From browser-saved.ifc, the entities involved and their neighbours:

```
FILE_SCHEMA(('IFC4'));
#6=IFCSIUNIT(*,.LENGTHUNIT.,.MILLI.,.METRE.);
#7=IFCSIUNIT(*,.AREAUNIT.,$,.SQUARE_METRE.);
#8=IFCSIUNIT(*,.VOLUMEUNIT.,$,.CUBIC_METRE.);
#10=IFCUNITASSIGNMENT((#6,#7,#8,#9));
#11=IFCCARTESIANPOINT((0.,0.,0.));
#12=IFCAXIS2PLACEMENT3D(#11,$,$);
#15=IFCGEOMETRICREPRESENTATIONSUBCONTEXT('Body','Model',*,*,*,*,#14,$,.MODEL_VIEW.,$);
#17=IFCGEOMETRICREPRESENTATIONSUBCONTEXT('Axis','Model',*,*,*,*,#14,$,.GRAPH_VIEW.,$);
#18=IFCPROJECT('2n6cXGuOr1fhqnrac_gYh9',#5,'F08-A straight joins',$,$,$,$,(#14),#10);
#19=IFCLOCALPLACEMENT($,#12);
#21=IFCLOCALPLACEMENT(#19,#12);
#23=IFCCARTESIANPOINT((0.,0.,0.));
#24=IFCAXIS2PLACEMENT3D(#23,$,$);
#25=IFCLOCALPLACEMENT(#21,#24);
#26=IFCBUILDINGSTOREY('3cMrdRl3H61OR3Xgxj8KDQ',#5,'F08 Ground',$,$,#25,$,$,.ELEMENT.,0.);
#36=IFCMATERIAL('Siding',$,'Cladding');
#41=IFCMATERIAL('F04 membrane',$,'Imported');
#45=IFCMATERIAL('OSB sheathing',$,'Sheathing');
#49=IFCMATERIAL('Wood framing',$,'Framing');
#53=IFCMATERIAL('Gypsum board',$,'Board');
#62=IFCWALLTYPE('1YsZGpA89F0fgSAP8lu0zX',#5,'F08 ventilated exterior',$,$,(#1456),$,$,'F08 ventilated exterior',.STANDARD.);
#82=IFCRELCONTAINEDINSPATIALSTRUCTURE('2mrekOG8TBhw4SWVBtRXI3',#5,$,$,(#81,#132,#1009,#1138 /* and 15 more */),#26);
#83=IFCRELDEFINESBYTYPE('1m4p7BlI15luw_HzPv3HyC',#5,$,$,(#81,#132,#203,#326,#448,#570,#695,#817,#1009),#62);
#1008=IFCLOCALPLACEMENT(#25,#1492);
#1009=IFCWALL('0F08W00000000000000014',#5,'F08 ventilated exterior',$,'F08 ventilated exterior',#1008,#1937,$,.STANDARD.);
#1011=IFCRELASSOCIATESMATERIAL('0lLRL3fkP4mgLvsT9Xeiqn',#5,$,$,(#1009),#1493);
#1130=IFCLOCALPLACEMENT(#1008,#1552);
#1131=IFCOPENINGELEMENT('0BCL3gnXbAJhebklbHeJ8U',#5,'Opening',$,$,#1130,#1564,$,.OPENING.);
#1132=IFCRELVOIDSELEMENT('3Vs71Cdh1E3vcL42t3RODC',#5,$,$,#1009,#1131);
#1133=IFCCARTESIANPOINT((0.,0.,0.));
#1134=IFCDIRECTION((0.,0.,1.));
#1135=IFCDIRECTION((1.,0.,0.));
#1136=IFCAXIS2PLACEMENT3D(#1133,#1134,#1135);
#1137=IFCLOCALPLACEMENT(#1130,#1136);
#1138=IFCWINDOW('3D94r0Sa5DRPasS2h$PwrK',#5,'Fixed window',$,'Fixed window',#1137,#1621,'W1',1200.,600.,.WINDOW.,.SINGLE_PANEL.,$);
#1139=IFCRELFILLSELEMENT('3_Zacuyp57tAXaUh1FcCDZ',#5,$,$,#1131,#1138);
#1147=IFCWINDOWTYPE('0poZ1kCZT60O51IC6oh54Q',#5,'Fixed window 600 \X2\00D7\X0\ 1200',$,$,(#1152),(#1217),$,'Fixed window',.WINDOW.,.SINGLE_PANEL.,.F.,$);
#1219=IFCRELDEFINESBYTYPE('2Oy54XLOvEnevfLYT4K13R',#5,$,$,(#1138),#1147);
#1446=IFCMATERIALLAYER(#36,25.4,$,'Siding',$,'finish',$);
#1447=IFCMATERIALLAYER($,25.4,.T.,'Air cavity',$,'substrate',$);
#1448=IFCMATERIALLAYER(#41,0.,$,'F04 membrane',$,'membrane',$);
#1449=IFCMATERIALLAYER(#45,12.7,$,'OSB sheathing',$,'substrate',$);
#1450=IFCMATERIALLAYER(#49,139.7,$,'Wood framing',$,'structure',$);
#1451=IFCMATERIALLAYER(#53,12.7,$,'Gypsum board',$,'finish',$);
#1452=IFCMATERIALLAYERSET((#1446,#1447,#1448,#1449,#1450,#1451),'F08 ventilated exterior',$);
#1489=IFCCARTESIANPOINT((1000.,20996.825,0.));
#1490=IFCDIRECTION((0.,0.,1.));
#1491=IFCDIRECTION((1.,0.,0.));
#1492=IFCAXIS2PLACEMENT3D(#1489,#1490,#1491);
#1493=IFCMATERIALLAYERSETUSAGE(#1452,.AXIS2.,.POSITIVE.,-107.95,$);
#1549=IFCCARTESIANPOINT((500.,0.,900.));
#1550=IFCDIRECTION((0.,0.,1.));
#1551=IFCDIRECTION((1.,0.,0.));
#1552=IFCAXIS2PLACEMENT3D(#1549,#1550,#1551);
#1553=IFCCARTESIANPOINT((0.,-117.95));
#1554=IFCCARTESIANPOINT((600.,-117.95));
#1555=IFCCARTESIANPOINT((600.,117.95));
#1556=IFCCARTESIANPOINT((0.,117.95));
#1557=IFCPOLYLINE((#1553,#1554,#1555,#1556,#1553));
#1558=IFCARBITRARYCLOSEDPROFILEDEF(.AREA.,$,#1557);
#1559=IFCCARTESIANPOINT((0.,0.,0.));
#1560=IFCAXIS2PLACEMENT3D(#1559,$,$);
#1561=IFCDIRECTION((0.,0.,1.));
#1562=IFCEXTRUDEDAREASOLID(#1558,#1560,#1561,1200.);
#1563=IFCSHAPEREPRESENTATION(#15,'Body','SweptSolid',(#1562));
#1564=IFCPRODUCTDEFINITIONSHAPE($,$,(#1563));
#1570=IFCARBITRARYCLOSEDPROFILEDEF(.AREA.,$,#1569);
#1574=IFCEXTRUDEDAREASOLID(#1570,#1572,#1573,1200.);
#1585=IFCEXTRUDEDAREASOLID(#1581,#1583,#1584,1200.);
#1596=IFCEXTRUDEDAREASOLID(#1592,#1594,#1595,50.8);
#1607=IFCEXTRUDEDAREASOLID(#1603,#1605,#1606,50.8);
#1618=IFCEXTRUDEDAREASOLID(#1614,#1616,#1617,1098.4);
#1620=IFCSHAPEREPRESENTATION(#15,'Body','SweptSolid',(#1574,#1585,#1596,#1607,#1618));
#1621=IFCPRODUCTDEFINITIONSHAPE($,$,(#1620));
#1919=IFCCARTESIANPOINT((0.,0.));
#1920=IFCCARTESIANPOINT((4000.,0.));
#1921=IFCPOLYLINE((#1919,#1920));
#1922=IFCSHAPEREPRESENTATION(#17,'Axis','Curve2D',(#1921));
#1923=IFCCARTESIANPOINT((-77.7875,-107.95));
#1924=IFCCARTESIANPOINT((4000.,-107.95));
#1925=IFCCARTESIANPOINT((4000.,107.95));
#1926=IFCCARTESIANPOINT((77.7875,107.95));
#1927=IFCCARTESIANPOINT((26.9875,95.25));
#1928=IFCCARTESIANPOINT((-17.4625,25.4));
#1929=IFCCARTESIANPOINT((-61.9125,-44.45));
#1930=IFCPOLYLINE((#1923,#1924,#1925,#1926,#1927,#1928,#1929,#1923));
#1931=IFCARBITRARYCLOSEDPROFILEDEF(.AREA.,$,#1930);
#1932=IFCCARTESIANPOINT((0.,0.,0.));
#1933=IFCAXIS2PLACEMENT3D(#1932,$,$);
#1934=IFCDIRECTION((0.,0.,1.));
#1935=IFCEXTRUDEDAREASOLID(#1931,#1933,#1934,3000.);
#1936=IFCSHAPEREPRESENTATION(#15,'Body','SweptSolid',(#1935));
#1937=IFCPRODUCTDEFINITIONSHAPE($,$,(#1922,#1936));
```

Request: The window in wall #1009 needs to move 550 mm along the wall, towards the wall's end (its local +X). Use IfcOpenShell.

```python
import ifcopenshell
import ifcopenshell.api.geometry
import ifcopenshell.util.placement
import ifcopenshell.util.unit

model = ifcopenshell.open("browser-saved.ifc")
unit_scale = ifcopenshell.util.unit.calculate_unit_scale(model)

window = model.by_id(1138)
opening = window.FillsVoids[0].RelatingOpeningElement
wall = opening.VoidsElements[0].RelatingBuildingElement

wall_matrix = ifcopenshell.util.placement.get_local_placement(wall.ObjectPlacement)
shift = wall_matrix[:3, 0] * 0.55 / unit_scale
before = ifcopenshell.util.placement.get_local_placement(window.ObjectPlacement)[:3, 3].copy()

# The window is placed relative to its opening, so it follows when the opening moves.
matrix = ifcopenshell.util.placement.get_local_placement(opening.ObjectPlacement)
matrix[:3, 3] += shift
ifcopenshell.api.geometry.edit_object_placement(
    model, product=opening, matrix=matrix, is_si=False, should_transform_children=True
)

after = ifcopenshell.util.placement.get_local_placement(window.ObjectPlacement)[:3, 3]
print("window moved by", (after - before).round(3) + 0.0)

model.write("browser-saved_edited.ifc")
```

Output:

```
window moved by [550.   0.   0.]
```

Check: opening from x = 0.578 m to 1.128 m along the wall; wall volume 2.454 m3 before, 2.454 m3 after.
